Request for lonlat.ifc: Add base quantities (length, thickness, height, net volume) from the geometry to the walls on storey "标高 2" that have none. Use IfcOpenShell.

First a look at what the model holds.

```python
import ifcopenshell
import ifcopenshell.util.element
import ifcopenshell.util.unit

model = ifcopenshell.open("lonlat.ifc")
print(model.schema)
for unit_type in ("LENGTHUNIT", "AREAUNIT", "VOLUMEUNIT"):
    print(unit_type, ifcopenshell.util.unit.calculate_unit_scale(model, unit_type))
storey = next(s for s in model.by_type("IfcBuildingStorey") if s.Name == "标高 2")
walls = [e for e in ifcopenshell.util.element.get_decomposition(storey) if e.is_a("IfcWall")]
for e in sorted(walls, key=lambda e: e.id()):
    print(e.id(), e.is_a(), e.Name, list(ifcopenshell.util.element.get_psets(e, qtos_only=True)), sep=" | ")
```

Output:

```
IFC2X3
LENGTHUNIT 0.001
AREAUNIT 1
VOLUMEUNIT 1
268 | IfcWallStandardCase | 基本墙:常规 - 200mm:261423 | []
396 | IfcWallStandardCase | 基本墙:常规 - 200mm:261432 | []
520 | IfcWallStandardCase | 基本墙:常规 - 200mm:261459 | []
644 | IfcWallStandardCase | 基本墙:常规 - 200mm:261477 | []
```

```python
import ifcopenshell
import ifcopenshell.api.pset
import ifcopenshell.geom
import ifcopenshell.util.element
import ifcopenshell.util.shape
import ifcopenshell.util.unit

model = ifcopenshell.open("lonlat.ifc")
unit_scale = ifcopenshell.util.unit.calculate_unit_scale(model)
volume_scale = ifcopenshell.util.unit.calculate_unit_scale(model, "VOLUMEUNIT")
settings = ifcopenshell.geom.settings()

storey = next(s for s in model.by_type("IfcBuildingStorey") if s.Name == "标高 2")
walls = [e for e in ifcopenshell.util.element.get_decomposition(storey) if e.is_a("IfcWall")]

for e in sorted(walls, key=lambda e: e.id()):
    if ifcopenshell.util.element.get_psets(e, qtos_only=True, should_inherit=False):
        continue
    # Geometry comes back in metres, in the element's own axes.
    shape = ifcopenshell.geom.create_shape(settings, e)
    values = {
        "Length": ifcopenshell.util.shape.get_x(shape.geometry) / unit_scale,
        "Width": ifcopenshell.util.shape.get_y(shape.geometry) / unit_scale,
        "Height": ifcopenshell.util.shape.get_z(shape.geometry) / unit_scale,
        "NetVolume": ifcopenshell.util.shape.get_volume(shape.geometry) / volume_scale,
    }
    qto = ifcopenshell.api.pset.add_qto(model, product=e, name="BaseQuantities")
    ifcopenshell.api.pset.edit_qto(model, qto=qto, properties=values)
    print(e.id(), {k: round(v, 3) for k, v in values.items()})

model.write("lonlat_rev.ifc")
```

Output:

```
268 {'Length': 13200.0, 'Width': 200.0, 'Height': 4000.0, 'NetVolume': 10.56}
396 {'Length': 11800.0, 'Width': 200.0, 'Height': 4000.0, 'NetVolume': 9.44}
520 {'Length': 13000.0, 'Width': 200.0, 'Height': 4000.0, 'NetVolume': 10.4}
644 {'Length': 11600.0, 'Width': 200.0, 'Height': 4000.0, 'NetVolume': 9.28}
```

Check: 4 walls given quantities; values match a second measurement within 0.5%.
